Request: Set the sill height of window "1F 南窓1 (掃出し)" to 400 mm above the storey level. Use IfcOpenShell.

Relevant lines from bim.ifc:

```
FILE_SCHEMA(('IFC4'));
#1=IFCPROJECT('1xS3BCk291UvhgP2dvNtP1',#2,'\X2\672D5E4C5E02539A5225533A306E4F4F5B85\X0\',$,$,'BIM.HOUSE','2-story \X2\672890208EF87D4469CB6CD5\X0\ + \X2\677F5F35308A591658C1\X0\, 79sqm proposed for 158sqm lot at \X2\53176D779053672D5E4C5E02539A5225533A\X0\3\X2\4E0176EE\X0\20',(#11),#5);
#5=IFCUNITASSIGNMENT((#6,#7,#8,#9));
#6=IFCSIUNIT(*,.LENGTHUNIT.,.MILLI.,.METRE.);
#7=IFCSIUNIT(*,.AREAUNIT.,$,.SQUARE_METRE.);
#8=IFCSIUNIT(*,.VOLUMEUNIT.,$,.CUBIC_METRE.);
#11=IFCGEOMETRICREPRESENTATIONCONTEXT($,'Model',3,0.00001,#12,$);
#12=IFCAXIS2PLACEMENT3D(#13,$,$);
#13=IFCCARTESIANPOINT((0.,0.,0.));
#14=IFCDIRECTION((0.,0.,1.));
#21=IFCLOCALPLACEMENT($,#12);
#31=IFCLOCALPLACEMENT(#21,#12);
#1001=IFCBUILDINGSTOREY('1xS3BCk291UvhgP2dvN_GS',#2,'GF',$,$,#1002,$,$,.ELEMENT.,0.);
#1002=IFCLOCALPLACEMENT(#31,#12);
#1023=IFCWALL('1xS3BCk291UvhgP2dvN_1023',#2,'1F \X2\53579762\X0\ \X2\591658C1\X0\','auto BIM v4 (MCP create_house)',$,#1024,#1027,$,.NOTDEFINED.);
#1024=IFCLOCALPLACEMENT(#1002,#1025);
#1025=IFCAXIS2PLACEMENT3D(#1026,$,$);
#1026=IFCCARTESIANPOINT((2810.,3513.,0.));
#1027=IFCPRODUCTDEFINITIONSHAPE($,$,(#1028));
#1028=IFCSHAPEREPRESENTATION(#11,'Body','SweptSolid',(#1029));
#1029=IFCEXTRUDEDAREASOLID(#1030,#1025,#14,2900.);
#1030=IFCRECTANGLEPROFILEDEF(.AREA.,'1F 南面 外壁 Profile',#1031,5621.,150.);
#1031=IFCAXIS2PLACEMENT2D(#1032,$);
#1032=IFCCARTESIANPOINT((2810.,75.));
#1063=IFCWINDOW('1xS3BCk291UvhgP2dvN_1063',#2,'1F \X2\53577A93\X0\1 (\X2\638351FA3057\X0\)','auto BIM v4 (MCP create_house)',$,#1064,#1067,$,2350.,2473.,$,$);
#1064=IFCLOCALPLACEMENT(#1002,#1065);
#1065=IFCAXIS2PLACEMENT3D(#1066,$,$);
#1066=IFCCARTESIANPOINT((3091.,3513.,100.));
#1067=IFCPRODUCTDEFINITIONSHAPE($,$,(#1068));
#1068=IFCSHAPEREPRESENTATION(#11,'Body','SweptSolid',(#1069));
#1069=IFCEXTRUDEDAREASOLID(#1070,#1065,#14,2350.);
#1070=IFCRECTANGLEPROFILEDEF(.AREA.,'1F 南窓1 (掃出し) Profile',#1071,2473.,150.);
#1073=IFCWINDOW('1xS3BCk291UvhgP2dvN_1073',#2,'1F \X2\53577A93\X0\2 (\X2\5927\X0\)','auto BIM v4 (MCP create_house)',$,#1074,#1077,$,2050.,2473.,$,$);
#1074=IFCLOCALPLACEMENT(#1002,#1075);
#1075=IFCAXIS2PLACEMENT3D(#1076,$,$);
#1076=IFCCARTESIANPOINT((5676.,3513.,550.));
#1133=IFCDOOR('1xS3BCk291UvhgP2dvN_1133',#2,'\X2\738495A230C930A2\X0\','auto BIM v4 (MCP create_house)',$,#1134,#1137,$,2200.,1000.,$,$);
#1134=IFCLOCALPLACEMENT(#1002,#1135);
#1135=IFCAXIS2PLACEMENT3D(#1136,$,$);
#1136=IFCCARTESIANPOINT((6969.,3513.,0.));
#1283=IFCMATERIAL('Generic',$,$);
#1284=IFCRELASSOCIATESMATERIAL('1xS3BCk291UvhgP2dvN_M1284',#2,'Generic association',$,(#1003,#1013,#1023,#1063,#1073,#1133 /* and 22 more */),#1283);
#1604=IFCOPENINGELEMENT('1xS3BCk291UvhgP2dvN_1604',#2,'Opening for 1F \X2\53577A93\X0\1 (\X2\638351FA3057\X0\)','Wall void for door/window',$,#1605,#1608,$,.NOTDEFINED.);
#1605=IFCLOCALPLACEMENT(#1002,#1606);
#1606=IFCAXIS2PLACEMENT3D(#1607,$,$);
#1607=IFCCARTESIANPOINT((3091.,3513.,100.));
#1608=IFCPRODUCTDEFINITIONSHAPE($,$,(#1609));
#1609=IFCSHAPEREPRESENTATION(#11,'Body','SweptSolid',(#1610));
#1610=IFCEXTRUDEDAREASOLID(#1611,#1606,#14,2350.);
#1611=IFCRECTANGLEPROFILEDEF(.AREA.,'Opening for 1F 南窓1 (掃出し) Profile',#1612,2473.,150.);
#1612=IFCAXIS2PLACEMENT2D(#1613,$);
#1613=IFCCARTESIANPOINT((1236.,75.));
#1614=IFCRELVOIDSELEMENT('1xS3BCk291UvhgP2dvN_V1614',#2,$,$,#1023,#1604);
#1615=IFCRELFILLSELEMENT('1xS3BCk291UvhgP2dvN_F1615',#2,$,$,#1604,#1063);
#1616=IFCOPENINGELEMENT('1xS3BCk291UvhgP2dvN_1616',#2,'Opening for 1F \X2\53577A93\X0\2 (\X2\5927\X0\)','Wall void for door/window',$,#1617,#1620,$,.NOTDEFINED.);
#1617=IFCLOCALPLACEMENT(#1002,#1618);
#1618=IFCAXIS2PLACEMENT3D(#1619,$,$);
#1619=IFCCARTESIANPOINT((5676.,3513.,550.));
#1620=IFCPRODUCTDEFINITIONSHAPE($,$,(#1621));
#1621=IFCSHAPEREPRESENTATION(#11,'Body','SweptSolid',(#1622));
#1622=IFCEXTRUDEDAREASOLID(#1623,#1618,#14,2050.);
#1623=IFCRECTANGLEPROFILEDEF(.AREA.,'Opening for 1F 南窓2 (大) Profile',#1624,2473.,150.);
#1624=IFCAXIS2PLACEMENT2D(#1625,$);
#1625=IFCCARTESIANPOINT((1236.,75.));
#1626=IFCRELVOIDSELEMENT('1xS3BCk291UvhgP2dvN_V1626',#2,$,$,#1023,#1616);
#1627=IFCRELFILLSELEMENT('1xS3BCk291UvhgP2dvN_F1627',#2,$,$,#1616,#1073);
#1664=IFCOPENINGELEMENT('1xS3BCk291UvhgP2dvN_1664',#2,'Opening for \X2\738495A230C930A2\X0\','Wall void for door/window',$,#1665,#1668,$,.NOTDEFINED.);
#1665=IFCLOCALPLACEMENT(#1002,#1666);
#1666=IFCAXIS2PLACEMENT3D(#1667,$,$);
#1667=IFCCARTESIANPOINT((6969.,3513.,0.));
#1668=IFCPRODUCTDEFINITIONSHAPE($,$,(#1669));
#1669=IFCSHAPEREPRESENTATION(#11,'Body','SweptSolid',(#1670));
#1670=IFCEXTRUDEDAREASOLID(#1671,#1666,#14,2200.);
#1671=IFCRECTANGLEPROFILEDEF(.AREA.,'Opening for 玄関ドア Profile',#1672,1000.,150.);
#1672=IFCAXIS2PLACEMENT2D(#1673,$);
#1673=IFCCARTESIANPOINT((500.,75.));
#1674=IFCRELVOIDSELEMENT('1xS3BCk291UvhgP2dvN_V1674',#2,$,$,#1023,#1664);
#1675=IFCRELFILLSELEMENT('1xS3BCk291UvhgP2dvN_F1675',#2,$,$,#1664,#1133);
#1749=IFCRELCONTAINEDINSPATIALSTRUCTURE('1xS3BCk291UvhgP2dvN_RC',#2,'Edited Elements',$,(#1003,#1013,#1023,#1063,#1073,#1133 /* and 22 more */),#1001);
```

```python
import numpy as np
import ifcopenshell
import ifcopenshell.api.geometry
import ifcopenshell.geom
import ifcopenshell.util.element
import ifcopenshell.util.placement
import ifcopenshell.util.shape
import ifcopenshell.util.unit

model = ifcopenshell.open("bim.ifc")
unit_scale = ifcopenshell.util.unit.calculate_unit_scale(model)

window = model.by_id(1063)
opening = window.FillsVoids[0].RelatingOpeningElement
storey = ifcopenshell.util.element.get_container(window, ifc_class="IfcBuildingStorey")
level = ifcopenshell.util.placement.get_local_placement(storey.ObjectPlacement)[2, 3]

# The opening's origin need not be at the sill, so measure its lowest point.
shape = ifcopenshell.geom.create_shape(ifcopenshell.geom.settings(), opening)
bottom = ifcopenshell.util.shape.get_shape_bottom_elevation(shape, shape.geometry) / unit_scale
dz = level + 0.4 / unit_scale - bottom

shift = np.array([0.0, 0.0, dz])
# The window is not placed relative to its opening, so move both.
for product in (opening, window):
    matrix = ifcopenshell.util.placement.get_local_placement(product.ObjectPlacement)
    matrix[:3, 3] += shift
    ifcopenshell.api.geometry.edit_object_placement(model, product=product, matrix=matrix, is_si=False)

print(f"moved by {dz * unit_scale:+.3f} m")

model.write("bim_v2.ifc")
```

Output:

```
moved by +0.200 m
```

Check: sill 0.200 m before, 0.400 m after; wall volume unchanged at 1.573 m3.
